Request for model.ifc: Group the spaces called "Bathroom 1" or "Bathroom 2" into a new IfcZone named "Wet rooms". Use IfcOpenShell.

First a look at what the model holds.

```python
import ifcopenshell

model = ifcopenshell.open("model.ifc")
print(model.schema)
seen = {}
for space in model.by_type("IfcSpace"):
    seen[space.LongName] = seen.get(space.LongName, 0) + 1
for name, count in sorted(seen.items(), key=str):
    print(count, "x", name)
print("zones:", [z.Name for z in model.by_type("IfcZone")][:20])
```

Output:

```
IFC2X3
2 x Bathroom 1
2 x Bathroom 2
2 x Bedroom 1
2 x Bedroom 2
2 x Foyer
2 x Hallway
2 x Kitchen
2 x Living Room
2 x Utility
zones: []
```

```python
import ifcopenshell
import ifcopenshell.api.group
import ifcopenshell.api.root

model = ifcopenshell.open("model.ifc")

names = {"Bathroom 1", "Bathroom 2"}
spaces = [s for s in model.by_type("IfcSpace") if s.LongName in names]

zone = ifcopenshell.api.root.create_entity(model, ifc_class="IfcZone", name="Wet rooms")
ifcopenshell.api.group.assign_group(model, products=spaces, group=zone)
print(len(spaces), "spaces in", zone.Name)

model.write("model_updated.ifc")
```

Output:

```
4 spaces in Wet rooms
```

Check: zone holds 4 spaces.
